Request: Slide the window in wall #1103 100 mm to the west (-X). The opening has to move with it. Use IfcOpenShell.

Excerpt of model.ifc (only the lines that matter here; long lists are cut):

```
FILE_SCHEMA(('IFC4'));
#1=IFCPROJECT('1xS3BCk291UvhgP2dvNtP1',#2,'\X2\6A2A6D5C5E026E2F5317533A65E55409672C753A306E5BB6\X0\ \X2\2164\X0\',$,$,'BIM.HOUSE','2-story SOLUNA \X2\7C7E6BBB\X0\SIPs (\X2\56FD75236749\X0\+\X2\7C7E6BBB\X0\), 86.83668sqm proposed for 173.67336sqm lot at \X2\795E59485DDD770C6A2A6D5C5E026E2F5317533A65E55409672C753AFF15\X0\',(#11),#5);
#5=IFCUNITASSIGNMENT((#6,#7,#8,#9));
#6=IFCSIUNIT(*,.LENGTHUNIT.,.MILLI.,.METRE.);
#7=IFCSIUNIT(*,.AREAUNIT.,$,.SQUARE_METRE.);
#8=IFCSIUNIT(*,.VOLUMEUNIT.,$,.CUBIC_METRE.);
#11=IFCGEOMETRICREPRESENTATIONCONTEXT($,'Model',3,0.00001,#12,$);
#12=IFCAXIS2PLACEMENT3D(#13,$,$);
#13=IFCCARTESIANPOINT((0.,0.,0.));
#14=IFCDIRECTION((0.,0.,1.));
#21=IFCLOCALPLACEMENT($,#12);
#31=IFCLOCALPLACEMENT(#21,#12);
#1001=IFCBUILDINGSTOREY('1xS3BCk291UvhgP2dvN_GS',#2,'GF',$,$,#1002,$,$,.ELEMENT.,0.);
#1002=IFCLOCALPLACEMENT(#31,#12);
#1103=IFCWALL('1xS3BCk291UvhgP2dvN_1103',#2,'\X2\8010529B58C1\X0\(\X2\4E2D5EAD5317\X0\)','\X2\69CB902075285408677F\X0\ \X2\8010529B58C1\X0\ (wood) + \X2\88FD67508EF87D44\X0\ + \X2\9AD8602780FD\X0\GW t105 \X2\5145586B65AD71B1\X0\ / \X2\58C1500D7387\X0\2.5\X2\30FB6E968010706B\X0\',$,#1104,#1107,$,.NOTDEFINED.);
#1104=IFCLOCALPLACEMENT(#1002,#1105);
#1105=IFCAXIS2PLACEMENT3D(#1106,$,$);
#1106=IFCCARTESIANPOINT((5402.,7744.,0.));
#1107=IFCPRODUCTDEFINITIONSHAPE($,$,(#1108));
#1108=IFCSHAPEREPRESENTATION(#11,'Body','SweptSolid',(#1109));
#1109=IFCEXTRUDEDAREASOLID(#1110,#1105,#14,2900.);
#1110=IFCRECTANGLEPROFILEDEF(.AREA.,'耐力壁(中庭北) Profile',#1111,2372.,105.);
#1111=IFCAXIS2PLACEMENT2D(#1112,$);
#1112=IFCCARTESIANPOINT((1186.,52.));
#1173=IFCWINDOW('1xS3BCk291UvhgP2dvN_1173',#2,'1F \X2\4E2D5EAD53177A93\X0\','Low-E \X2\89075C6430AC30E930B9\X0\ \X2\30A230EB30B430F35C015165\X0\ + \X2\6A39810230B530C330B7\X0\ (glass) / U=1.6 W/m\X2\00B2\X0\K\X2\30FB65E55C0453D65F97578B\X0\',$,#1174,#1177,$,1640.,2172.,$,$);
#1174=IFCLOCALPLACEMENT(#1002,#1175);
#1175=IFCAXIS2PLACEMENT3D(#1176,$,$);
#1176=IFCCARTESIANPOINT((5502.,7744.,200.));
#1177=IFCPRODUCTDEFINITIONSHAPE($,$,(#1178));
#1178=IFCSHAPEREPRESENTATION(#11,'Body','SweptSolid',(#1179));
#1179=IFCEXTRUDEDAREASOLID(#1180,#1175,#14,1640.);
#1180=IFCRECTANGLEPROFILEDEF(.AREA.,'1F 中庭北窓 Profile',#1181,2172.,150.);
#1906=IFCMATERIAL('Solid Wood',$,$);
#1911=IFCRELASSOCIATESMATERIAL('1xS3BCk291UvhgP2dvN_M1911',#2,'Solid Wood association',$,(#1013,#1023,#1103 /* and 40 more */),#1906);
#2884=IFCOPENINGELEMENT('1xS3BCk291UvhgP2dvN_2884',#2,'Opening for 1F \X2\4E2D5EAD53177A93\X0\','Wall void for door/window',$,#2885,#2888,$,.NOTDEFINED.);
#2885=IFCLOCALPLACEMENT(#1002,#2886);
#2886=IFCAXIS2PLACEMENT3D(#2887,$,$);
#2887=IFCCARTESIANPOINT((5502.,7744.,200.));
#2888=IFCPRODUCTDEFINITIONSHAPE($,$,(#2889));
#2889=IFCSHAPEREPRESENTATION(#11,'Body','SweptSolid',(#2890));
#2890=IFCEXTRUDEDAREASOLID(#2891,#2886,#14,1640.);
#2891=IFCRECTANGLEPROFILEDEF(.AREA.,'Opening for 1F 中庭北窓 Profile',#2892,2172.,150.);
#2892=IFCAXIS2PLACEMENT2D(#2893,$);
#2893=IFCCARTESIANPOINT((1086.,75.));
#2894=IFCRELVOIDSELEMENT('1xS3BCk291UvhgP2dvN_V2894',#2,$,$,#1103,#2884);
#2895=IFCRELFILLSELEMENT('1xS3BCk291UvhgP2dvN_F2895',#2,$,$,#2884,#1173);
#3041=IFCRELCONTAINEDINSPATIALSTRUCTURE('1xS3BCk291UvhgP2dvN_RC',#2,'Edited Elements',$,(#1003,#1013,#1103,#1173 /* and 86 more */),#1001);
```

```python
import ifcopenshell
import ifcopenshell.api.geometry
import ifcopenshell.util.placement

model = ifcopenshell.open("model.ifc")

window = model.by_guid("1xS3BCk291UvhgP2dvN_1173")
opening = window.FillsVoids[0].RelatingOpeningElement
wall = opening.VoidsElements[0].RelatingBuildingElement

wall_matrix = ifcopenshell.util.placement.get_local_placement(wall.ObjectPlacement)
shift = wall_matrix[:3, 0] * -100.0
before = ifcopenshell.util.placement.get_local_placement(window.ObjectPlacement)[:3, 3].copy()

# The window is not placed relative to its opening, so move both.
for product in (opening, window):
    matrix = ifcopenshell.util.placement.get_local_placement(product.ObjectPlacement)
    matrix[:3, 3] += shift
    ifcopenshell.api.geometry.edit_object_placement(model, product=product, matrix=matrix, is_si=False)

after = ifcopenshell.util.placement.get_local_placement(window.ObjectPlacement)[:3, 3]
print("window moved by", (after - before).round(3) + 0.0)

model.write("model_updated.ifc")
```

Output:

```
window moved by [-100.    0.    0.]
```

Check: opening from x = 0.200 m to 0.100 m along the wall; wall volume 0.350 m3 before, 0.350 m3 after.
